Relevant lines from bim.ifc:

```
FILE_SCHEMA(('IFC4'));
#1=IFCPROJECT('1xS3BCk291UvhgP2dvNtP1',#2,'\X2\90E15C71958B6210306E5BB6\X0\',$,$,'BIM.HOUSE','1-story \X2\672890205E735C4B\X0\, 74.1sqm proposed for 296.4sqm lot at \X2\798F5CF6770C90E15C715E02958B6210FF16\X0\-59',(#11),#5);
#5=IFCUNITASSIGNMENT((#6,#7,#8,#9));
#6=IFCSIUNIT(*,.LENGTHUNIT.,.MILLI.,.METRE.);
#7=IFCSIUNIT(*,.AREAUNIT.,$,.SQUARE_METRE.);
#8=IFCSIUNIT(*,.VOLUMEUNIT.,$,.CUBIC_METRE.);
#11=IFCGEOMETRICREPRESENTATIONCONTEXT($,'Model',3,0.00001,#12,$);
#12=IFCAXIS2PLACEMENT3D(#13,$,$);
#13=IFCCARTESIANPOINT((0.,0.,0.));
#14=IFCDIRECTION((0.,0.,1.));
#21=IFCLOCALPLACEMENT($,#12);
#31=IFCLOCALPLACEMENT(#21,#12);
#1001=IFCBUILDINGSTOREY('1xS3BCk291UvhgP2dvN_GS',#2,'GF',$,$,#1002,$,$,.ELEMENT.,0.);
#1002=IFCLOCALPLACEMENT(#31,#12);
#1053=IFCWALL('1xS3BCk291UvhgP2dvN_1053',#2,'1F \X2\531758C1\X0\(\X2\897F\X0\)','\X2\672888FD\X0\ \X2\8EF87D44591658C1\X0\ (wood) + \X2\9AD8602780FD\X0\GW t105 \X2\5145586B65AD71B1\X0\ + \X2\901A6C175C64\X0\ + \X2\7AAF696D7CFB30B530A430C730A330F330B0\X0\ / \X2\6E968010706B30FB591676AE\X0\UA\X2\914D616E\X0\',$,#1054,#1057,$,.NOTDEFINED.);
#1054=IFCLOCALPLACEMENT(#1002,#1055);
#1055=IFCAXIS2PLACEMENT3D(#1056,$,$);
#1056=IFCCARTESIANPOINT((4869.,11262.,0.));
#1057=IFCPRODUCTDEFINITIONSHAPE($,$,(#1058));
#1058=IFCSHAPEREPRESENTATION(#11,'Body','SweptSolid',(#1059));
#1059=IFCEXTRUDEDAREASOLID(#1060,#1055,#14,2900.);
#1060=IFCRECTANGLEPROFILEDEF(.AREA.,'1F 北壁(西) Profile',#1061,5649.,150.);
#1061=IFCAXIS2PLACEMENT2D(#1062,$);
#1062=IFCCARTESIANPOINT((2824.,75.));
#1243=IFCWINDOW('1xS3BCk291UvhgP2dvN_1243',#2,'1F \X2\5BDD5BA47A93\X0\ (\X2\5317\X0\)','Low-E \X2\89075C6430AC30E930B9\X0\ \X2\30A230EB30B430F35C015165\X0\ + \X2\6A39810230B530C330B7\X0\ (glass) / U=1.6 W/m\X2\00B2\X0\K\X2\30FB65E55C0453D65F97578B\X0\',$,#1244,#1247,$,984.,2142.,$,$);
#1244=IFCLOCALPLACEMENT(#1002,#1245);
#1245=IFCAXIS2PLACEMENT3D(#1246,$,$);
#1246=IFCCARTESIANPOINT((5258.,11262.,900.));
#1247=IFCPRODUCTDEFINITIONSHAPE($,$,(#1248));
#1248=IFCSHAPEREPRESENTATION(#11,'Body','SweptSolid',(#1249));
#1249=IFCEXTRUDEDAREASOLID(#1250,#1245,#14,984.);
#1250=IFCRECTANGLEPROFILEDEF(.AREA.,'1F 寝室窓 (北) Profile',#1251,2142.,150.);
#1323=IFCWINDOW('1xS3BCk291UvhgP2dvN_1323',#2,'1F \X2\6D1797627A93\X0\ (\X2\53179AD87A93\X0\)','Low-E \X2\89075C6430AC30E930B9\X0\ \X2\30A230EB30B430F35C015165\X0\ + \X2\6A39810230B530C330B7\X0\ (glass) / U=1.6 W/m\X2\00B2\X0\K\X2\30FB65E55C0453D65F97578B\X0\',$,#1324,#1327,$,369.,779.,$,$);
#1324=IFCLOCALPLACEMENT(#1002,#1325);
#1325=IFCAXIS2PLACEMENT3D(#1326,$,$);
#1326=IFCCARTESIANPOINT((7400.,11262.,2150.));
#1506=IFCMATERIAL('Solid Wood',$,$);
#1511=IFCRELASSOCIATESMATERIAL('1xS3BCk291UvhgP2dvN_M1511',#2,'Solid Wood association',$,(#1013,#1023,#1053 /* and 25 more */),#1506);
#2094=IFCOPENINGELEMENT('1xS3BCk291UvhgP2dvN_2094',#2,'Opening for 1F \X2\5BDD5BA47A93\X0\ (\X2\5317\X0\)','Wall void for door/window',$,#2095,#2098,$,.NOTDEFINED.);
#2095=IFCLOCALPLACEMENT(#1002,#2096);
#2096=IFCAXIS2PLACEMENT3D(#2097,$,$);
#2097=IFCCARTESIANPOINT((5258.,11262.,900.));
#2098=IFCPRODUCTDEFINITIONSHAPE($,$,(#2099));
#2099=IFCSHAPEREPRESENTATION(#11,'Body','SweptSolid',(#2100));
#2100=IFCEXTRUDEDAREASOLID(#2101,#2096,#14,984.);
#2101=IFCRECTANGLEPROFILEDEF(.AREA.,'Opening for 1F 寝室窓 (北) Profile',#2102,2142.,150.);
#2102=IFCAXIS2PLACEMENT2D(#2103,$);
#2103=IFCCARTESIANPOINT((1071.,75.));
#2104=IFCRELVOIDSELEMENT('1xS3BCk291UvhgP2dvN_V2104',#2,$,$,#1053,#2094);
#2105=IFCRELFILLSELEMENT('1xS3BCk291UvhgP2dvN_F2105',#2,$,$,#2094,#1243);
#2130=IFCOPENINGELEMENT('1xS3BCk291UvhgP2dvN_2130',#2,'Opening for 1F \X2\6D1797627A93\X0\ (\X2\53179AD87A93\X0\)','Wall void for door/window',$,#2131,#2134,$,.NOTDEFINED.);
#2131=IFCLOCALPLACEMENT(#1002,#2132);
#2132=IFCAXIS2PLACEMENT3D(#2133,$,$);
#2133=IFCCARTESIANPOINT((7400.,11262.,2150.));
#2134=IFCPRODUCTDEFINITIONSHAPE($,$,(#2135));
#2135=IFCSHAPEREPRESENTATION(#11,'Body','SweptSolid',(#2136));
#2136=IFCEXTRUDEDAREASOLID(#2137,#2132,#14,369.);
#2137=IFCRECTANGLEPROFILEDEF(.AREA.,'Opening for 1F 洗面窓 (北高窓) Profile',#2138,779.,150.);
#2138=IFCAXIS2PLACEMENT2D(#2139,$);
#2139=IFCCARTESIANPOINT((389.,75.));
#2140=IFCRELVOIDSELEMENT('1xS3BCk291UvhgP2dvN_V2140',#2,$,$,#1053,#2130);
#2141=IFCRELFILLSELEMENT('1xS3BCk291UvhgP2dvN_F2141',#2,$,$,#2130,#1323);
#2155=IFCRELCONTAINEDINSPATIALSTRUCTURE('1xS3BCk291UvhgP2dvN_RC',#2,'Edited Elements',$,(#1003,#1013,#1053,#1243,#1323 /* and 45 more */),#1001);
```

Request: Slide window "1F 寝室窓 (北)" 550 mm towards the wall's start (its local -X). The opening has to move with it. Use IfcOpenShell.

```python
import ifcopenshell
import ifcopenshell.api.geometry
import ifcopenshell.util.placement
import ifcopenshell.util.unit

model = ifcopenshell.open("bim.ifc")
unit_scale = ifcopenshell.util.unit.calculate_unit_scale(model)

window = model.by_guid("1xS3BCk291UvhgP2dvN_1243")
opening = window.FillsVoids[0].RelatingOpeningElement
wall = opening.VoidsElements[0].RelatingBuildingElement

wall_matrix = ifcopenshell.util.placement.get_local_placement(wall.ObjectPlacement)
shift = wall_matrix[:3, 0] * -0.55 / unit_scale
before = ifcopenshell.util.placement.get_local_placement(window.ObjectPlacement)[:3, 3].copy()

# The window is not placed relative to its opening, so move both.
for product in (opening, window):
    matrix = ifcopenshell.util.placement.get_local_placement(product.ObjectPlacement)
    matrix[:3, 3] += shift
    ifcopenshell.api.geometry.edit_object_placement(model, product=product, matrix=matrix, is_si=False)

after = ifcopenshell.util.placement.get_local_placement(window.ObjectPlacement)[:3, 3]
print("window moved by", (after - before).round(3) + 0.0)

model.write("bim_updated.ifc")
```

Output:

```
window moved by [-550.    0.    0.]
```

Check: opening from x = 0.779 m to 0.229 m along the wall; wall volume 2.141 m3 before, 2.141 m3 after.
